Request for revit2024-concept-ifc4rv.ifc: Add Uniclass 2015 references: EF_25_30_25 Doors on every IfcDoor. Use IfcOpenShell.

First a look at what the model holds.

```python
import ifcopenshell

model = ifcopenshell.open("revit2024-concept-ifc4rv.ifc")
print(model.schema)
print("classifications:", [c.Name for c in model.by_type("IfcClassification")])
for ifc_class in ("IfcDoor", "IfcRoof", "IfcStair", "IfcWall", "IfcWindow"):
    print(ifc_class, len(model.by_type(ifc_class)))
```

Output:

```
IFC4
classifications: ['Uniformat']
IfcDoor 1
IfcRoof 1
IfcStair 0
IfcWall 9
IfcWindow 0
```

```python
import ifcopenshell
import ifcopenshell.api.classification

model = ifcopenshell.open("revit2024-concept-ifc4rv.ifc")

system = ifcopenshell.api.classification.add_classification(model, classification="Uniclass 2015")

codes = {
    "IfcDoor": ("EF_25_30_25", "Doors"),
}
for ifc_class, (code, name) in codes.items():
    products = model.by_type(ifc_class)
    ifcopenshell.api.classification.add_reference(
        model, products=products, classification=system, identification=code, name=name
    )
    print(code, len(products))

model.write("revit2024-concept-ifc4rv_rev.ifc")
```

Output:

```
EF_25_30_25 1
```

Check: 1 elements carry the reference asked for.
